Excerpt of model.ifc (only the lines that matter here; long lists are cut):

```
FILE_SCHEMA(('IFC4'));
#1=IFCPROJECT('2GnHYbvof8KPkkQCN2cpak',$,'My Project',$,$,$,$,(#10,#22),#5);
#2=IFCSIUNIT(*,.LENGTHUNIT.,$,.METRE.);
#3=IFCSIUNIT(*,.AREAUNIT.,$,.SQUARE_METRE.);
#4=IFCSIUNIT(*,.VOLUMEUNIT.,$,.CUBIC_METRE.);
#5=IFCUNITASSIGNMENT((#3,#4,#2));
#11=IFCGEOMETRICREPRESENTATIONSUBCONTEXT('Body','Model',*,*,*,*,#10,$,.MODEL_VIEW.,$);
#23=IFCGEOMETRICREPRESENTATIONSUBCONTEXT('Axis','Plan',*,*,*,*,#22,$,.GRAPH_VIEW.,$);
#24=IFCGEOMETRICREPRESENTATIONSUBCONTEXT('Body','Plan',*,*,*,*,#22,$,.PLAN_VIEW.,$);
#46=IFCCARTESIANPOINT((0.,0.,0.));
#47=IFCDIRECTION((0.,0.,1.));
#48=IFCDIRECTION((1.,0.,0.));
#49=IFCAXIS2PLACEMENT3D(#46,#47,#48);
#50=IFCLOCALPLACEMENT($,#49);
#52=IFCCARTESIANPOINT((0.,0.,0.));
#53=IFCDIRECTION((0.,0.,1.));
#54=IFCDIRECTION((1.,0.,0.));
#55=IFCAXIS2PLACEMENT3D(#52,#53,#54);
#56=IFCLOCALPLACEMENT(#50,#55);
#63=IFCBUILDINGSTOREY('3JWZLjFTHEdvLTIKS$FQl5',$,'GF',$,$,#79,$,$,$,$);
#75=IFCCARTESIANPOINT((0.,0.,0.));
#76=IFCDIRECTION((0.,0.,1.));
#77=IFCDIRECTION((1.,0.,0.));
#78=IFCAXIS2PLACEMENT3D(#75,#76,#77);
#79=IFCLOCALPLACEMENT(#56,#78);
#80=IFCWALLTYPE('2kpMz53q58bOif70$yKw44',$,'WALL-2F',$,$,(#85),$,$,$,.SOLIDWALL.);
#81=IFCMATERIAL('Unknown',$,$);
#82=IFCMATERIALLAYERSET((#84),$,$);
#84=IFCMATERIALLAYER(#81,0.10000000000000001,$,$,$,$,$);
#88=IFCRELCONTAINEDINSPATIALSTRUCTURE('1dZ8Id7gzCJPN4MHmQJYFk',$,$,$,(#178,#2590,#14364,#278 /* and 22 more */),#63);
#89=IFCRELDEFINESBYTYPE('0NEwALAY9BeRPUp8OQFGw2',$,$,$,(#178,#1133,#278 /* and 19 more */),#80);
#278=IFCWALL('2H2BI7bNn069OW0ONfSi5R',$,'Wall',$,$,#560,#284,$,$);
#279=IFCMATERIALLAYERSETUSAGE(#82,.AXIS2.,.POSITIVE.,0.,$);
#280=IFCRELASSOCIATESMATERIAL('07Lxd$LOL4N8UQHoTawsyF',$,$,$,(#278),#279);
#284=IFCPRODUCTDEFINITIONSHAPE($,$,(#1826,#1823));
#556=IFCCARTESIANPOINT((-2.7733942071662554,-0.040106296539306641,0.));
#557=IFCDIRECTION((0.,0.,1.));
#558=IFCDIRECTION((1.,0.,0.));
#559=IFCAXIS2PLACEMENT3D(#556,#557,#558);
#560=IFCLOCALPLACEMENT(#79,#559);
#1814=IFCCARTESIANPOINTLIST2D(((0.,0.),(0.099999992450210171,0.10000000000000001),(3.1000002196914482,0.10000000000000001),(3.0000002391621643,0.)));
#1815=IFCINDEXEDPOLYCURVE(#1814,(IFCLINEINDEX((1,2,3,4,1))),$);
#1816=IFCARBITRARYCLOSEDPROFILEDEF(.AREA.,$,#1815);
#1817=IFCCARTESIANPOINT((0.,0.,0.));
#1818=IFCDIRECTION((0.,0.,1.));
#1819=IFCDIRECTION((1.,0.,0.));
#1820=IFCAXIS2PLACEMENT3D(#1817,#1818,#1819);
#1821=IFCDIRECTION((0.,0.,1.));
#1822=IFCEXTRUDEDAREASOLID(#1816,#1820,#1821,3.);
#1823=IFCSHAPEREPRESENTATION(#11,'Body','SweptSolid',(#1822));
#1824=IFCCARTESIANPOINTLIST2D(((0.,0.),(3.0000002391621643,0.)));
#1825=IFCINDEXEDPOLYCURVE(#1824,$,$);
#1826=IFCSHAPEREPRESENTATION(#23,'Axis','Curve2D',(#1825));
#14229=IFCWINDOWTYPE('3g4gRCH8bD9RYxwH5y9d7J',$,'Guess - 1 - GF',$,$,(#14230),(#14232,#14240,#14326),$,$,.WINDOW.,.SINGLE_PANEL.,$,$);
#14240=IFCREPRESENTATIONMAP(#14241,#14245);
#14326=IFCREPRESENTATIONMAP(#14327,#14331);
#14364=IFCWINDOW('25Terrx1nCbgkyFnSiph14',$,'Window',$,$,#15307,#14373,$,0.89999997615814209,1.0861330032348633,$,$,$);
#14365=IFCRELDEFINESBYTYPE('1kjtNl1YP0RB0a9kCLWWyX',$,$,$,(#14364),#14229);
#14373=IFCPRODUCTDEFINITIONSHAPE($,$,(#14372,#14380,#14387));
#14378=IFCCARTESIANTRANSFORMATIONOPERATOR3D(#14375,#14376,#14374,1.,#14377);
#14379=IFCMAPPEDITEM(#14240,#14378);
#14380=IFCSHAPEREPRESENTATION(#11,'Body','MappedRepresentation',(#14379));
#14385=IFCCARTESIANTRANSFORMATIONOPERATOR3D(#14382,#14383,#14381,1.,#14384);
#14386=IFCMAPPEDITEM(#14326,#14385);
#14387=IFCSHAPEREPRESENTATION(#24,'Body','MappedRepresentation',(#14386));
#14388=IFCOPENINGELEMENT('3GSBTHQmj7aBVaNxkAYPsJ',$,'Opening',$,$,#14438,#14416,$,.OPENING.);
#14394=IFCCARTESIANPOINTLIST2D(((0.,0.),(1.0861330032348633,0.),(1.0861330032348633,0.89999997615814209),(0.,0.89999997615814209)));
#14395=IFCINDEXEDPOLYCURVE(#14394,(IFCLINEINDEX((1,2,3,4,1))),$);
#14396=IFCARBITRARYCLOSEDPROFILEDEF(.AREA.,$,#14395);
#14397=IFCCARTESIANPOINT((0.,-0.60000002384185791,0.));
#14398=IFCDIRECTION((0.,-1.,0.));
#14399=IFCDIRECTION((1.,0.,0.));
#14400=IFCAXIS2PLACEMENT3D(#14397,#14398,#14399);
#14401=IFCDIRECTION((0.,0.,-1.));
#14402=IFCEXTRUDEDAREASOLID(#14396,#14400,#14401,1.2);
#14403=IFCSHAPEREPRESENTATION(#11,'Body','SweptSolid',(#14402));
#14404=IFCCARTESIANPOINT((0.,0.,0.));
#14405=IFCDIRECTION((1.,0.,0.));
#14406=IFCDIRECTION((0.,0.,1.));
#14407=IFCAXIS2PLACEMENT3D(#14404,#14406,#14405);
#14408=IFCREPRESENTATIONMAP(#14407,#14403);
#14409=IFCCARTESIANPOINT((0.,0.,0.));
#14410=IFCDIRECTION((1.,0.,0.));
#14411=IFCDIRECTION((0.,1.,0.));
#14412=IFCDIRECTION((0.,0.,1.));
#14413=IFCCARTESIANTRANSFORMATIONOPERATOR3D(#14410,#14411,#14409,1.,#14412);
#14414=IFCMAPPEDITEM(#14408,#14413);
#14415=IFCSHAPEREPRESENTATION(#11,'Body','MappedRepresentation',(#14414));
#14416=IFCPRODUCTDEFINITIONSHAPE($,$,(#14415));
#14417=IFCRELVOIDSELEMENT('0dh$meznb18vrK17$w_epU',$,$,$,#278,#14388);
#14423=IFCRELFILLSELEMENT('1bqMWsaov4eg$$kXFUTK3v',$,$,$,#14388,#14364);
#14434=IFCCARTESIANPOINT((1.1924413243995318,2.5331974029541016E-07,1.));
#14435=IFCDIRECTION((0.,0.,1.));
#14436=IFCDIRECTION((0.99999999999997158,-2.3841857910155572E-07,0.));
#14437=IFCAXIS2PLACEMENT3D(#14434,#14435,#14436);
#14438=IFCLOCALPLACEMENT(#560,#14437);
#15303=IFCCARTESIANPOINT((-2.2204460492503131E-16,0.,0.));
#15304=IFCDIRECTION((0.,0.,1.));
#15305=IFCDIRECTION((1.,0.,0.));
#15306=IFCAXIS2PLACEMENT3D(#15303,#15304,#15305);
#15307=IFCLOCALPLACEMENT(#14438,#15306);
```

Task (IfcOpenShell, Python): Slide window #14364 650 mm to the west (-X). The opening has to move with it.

```python
import ifcopenshell
import ifcopenshell.api.geometry
import ifcopenshell.util.placement
import ifcopenshell.util.unit

model = ifcopenshell.open("model.ifc")
unit_scale = ifcopenshell.util.unit.calculate_unit_scale(model)

window = model.by_guid("25Terrx1nCbgkyFnSiph14")
opening = window.FillsVoids[0].RelatingOpeningElement
wall = opening.VoidsElements[0].RelatingBuildingElement

wall_matrix = ifcopenshell.util.placement.get_local_placement(wall.ObjectPlacement)
shift = wall_matrix[:3, 0] * -0.65 / unit_scale
before = ifcopenshell.util.placement.get_local_placement(window.ObjectPlacement)[:3, 3].copy()

# The window is placed relative to its opening, so it follows when the opening moves.
matrix = ifcopenshell.util.placement.get_local_placement(opening.ObjectPlacement)
matrix[:3, 3] += shift
ifcopenshell.api.geometry.edit_object_placement(
    model, product=opening, matrix=matrix, is_si=False, should_transform_children=True
)

after = ifcopenshell.util.placement.get_local_placement(window.ObjectPlacement)[:3, 3]
print("window moved by", (after - before).round(3) + 0.0)

model.write("model_v2.ifc")
```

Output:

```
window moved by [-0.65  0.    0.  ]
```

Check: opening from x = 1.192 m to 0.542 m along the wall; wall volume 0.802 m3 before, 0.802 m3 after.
